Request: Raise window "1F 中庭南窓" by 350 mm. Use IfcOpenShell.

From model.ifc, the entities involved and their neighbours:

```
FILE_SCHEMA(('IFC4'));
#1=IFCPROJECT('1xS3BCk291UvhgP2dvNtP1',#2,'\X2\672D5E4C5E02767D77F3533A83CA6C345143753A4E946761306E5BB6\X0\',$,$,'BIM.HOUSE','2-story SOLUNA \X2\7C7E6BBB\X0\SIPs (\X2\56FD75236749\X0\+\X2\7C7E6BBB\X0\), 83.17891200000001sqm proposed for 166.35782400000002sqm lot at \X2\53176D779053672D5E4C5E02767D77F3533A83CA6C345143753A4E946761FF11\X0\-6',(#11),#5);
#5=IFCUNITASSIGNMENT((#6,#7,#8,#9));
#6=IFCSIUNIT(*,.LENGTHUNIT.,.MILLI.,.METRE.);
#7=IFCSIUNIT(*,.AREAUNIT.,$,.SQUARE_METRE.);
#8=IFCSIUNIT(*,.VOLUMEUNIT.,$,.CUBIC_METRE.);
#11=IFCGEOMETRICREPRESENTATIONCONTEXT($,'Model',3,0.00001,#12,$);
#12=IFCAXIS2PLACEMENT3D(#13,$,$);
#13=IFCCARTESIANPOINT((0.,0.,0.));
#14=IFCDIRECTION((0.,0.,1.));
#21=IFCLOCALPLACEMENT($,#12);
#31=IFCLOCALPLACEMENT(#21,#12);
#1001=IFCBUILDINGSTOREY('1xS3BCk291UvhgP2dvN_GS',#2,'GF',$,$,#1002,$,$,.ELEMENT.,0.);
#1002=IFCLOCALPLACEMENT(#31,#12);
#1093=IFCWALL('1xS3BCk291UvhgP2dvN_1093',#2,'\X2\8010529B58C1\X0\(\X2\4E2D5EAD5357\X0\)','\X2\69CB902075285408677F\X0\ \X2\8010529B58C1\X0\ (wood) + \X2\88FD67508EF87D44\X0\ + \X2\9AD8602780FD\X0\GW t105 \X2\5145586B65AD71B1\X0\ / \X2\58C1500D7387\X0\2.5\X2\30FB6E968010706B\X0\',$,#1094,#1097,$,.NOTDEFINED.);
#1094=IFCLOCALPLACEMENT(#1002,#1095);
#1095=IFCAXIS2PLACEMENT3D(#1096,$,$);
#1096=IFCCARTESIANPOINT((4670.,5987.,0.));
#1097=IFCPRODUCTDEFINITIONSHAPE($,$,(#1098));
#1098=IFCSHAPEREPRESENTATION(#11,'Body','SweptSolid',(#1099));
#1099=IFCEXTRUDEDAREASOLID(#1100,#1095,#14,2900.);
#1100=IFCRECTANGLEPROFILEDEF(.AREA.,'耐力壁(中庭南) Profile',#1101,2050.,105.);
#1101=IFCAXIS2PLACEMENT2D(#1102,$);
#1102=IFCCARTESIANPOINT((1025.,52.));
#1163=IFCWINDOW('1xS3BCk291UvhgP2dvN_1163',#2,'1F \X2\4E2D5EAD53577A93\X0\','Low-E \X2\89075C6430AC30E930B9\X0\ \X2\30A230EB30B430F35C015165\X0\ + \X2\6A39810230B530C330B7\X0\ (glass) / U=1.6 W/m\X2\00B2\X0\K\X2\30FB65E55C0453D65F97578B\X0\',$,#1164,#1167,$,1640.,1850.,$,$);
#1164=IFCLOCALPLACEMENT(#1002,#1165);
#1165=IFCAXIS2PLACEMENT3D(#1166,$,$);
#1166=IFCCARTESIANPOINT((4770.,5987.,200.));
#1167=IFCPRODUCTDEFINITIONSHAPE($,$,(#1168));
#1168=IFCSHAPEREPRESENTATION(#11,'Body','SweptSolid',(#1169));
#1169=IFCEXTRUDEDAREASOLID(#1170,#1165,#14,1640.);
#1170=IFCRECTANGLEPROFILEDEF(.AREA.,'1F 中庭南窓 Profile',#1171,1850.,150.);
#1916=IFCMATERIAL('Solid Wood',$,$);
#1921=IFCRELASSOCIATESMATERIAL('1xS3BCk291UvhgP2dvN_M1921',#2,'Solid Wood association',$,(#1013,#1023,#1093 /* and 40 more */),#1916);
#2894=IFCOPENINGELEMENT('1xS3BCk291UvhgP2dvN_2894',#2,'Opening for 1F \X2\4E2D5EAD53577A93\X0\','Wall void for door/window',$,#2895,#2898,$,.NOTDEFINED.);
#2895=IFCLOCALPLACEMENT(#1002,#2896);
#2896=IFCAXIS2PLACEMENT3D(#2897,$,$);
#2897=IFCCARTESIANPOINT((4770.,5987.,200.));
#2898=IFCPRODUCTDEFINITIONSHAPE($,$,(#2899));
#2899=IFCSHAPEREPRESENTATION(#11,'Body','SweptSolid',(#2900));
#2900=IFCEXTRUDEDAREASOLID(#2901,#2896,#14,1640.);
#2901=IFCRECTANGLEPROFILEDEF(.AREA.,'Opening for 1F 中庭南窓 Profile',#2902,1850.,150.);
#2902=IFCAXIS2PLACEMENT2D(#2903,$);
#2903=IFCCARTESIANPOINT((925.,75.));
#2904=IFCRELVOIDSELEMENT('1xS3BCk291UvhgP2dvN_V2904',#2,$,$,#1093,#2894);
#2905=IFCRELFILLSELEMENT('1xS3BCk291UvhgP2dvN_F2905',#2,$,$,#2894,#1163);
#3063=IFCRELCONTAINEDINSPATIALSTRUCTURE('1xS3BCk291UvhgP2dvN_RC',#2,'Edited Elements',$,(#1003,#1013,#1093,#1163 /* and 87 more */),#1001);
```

```python
import numpy as np
import ifcopenshell
import ifcopenshell.api.geometry
import ifcopenshell.util.placement
import ifcopenshell.util.unit

model = ifcopenshell.open("model.ifc")
unit_scale = ifcopenshell.util.unit.calculate_unit_scale(model)

window = model.by_id(1163)
opening = window.FillsVoids[0].RelatingOpeningElement
dz = 350.0

shift = np.array([0.0, 0.0, dz])
# The window is not placed relative to its opening, so move both.
for product in (opening, window):
    matrix = ifcopenshell.util.placement.get_local_placement(product.ObjectPlacement)
    matrix[:3, 3] += shift
    ifcopenshell.api.geometry.edit_object_placement(model, product=product, matrix=matrix, is_si=False)

print(f"moved by {dz * unit_scale:+.3f} m")

model.write("model-out.ifc")
```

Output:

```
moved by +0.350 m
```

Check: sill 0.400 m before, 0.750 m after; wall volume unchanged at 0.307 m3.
